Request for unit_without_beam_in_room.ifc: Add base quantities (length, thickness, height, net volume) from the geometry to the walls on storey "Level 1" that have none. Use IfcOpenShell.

First a look at what the model holds.

```python
import ifcopenshell
import ifcopenshell.util.element
import ifcopenshell.util.unit

model = ifcopenshell.open("unit_without_beam_in_room.ifc")
print(model.schema)
for unit_type in ("LENGTHUNIT", "AREAUNIT", "VOLUMEUNIT"):
    print(unit_type, ifcopenshell.util.unit.calculate_unit_scale(model, unit_type))
storey = next(s for s in model.by_type("IfcBuildingStorey") if s.Name == "Level 1")
walls = [e for e in ifcopenshell.util.element.get_decomposition(storey) if e.is_a("IfcWall")]
for e in sorted(walls, key=lambda e: e.id()):
    print(e.id(), e.is_a(), e.Name, list(ifcopenshell.util.element.get_psets(e, qtos_only=True)), sep=" | ")
```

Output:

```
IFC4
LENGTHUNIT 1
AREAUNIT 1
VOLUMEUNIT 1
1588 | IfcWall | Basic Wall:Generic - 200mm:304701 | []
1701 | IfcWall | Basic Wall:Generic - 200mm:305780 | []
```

```python
import ifcopenshell
import ifcopenshell.api.pset
import ifcopenshell.geom
import ifcopenshell.util.element
import ifcopenshell.util.shape
import ifcopenshell.util.unit

model = ifcopenshell.open("unit_without_beam_in_room.ifc")
unit_scale = ifcopenshell.util.unit.calculate_unit_scale(model)
volume_scale = ifcopenshell.util.unit.calculate_unit_scale(model, "VOLUMEUNIT")
settings = ifcopenshell.geom.settings()

storey = next(s for s in model.by_type("IfcBuildingStorey") if s.Name == "Level 1")
walls = [e for e in ifcopenshell.util.element.get_decomposition(storey) if e.is_a("IfcWall")]

for e in sorted(walls, key=lambda e: e.id()):
    if ifcopenshell.util.element.get_psets(e, qtos_only=True, should_inherit=False):
        continue
    # Geometry comes back in metres, in the element's own axes.
    shape = ifcopenshell.geom.create_shape(settings, e)
    values = {
        "Length": ifcopenshell.util.shape.get_x(shape.geometry) / unit_scale,
        "Width": ifcopenshell.util.shape.get_y(shape.geometry) / unit_scale,
        "Height": ifcopenshell.util.shape.get_z(shape.geometry) / unit_scale,
        "NetVolume": ifcopenshell.util.shape.get_volume(shape.geometry) / volume_scale,
    }
    qto = ifcopenshell.api.pset.add_qto(model, product=e, name="Qto_WallBaseQuantities")
    ifcopenshell.api.pset.edit_qto(model, qto=qto, properties=values)
    print(e.id(), {k: round(v, 3) for k, v in values.items()})

model.write("unit_without_beam_in_room_rev.ifc")
```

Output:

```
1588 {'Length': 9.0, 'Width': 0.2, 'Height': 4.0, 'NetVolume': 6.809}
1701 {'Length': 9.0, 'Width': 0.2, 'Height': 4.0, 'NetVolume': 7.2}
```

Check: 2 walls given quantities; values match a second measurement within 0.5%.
